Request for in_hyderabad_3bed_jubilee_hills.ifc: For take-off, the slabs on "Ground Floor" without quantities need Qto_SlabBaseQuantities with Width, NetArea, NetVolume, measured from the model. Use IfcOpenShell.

First a look at what the model holds.

```python
import ifcopenshell
import ifcopenshell.util.element
import ifcopenshell.util.unit

model = ifcopenshell.open("in_hyderabad_3bed_jubilee_hills.ifc")
print(model.schema)
for unit_type in ("LENGTHUNIT", "AREAUNIT", "VOLUMEUNIT"):
    print(unit_type, ifcopenshell.util.unit.calculate_unit_scale(model, unit_type))
storey = next(s for s in model.by_type("IfcBuildingStorey") if s.Name == "Ground Floor")
slabs = [e for e in ifcopenshell.util.element.get_decomposition(storey) if e.is_a("IfcSlab")]
for e in sorted(slabs, key=lambda e: e.id()):
    print(e.id(), e.is_a(), e.Name, list(ifcopenshell.util.element.get_psets(e, qtos_only=True)), sep=" | ")
```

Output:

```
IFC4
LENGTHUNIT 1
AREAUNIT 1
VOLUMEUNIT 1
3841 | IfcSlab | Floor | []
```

```python
import ifcopenshell
import ifcopenshell.api.pset
import ifcopenshell.geom
import ifcopenshell.util.element
import ifcopenshell.util.shape
import ifcopenshell.util.unit

model = ifcopenshell.open("in_hyderabad_3bed_jubilee_hills.ifc")
unit_scale = ifcopenshell.util.unit.calculate_unit_scale(model)
area_scale = ifcopenshell.util.unit.calculate_unit_scale(model, "AREAUNIT")
volume_scale = ifcopenshell.util.unit.calculate_unit_scale(model, "VOLUMEUNIT")
settings = ifcopenshell.geom.settings()

storey = next(s for s in model.by_type("IfcBuildingStorey") if s.Name == "Ground Floor")
slabs = [e for e in ifcopenshell.util.element.get_decomposition(storey) if e.is_a("IfcSlab")]

for e in sorted(slabs, key=lambda e: e.id()):
    if ifcopenshell.util.element.get_psets(e, qtos_only=True, should_inherit=False):
        continue
    # Geometry comes back in metres, in the element's own axes.
    shape = ifcopenshell.geom.create_shape(settings, e)
    values = {
        "Width": ifcopenshell.util.shape.get_z(shape.geometry) / unit_scale,
        "NetArea": ifcopenshell.util.shape.get_footprint_area(shape.geometry) / area_scale,
        "NetVolume": ifcopenshell.util.shape.get_volume(shape.geometry) / volume_scale,
    }
    qto = ifcopenshell.api.pset.add_qto(model, product=e, name="Qto_SlabBaseQuantities")
    ifcopenshell.api.pset.edit_qto(model, qto=qto, properties=values)
    print(e.id(), {k: round(v, 3) for k, v in values.items()})

model.write("in_hyderabad_3bed_jubilee_hills_updated.ifc")
```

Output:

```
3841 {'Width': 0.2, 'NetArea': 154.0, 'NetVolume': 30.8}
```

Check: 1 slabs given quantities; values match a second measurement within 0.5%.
